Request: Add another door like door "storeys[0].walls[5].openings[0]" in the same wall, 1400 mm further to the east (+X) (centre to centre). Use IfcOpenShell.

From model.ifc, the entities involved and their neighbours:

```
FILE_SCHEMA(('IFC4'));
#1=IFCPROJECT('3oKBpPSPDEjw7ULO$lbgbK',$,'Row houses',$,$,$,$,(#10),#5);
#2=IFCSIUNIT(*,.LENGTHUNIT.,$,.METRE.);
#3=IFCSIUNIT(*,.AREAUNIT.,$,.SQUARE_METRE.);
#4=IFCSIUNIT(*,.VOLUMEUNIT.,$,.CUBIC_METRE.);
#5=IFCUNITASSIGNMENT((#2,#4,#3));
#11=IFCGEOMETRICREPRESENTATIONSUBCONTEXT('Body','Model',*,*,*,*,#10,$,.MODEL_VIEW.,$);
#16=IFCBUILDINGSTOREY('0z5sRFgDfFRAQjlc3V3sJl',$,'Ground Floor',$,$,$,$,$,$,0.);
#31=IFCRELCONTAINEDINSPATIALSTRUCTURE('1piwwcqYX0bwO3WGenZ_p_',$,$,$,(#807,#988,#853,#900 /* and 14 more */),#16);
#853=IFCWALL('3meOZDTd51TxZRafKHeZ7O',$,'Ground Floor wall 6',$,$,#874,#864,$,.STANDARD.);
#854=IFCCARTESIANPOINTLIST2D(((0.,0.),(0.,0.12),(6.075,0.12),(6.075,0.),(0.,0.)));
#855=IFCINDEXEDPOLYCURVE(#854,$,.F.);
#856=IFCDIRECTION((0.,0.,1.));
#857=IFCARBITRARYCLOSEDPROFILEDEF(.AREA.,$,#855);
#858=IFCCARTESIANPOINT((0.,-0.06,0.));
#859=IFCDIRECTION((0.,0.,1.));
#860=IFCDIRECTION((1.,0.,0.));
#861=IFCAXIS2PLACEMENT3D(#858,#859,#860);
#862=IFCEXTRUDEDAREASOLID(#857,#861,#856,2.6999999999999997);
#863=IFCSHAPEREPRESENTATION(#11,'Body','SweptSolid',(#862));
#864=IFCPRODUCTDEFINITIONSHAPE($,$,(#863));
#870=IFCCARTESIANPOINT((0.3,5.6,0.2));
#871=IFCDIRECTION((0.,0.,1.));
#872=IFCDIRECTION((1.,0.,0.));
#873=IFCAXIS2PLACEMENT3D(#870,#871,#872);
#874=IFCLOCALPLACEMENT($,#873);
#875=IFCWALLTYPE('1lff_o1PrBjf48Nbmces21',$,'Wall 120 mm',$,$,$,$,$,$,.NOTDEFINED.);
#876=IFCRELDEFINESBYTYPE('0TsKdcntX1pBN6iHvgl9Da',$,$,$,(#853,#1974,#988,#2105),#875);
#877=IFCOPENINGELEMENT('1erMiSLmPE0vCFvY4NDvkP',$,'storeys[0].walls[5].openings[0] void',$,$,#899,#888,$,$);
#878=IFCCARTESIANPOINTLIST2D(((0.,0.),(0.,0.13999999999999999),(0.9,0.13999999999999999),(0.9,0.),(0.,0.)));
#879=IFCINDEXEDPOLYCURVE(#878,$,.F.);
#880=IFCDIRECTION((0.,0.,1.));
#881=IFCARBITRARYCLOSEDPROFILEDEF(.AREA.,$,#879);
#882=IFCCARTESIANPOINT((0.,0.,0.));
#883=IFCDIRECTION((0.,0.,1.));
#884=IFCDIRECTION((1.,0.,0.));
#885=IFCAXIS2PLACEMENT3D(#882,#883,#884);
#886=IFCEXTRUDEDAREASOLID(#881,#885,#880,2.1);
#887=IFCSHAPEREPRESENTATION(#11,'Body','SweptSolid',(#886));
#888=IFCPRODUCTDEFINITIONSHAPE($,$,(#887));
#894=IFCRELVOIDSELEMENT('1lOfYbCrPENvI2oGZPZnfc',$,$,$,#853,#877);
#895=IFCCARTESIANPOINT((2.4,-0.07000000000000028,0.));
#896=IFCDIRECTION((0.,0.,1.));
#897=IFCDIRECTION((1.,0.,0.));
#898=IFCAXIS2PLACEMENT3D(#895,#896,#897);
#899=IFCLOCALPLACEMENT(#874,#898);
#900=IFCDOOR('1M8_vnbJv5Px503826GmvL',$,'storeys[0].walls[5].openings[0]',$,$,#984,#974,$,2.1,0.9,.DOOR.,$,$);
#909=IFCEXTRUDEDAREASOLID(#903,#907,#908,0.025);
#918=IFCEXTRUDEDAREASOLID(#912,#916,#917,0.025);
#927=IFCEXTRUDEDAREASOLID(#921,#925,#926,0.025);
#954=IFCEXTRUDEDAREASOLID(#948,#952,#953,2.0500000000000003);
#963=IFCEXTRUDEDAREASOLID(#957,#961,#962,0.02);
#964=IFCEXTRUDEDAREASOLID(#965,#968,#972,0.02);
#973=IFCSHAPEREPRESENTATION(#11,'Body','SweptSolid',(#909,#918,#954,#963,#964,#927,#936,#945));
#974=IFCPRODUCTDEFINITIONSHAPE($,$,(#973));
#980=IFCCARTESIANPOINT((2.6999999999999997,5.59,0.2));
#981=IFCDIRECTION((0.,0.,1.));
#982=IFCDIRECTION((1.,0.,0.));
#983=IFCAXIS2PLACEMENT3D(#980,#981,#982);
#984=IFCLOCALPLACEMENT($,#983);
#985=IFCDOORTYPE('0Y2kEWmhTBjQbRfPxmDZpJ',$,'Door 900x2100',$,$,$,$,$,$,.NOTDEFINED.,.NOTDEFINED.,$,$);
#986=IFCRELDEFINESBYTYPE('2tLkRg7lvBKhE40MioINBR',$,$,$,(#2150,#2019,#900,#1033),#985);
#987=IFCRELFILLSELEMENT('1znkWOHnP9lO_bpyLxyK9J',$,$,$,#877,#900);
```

```python
import ifcopenshell
import ifcopenshell.api.feature
import ifcopenshell.api.geometry
import ifcopenshell.api.root
import ifcopenshell.geom
import ifcopenshell.util.element
import ifcopenshell.util.placement
import ifcopenshell.util.shape

model = ifcopenshell.open("model.ifc")
settings = ifcopenshell.geom.settings()


def volume(element):
    """Net volume in cubic metres, openings subtracted."""
    shape = ifcopenshell.geom.create_shape(settings, element)
    return ifcopenshell.util.shape.get_volume(shape.geometry)


door = model.by_guid("1M8_vnbJv5Px503826GmvL")
opening = door.FillsVoids[0].RelatingOpeningElement
wall = opening.VoidsElements[0].RelatingBuildingElement
before = volume(wall)
shift = ifcopenshell.util.placement.get_local_placement(wall.ObjectPlacement)[:3, 0] * 1.4

# copy_class copies the void relationship, type, container and properties, but no geometry.
new_opening = ifcopenshell.api.root.copy_class(model, product=opening)
new_opening.Representation = ifcopenshell.util.element.copy_deep(
    model, opening.Representation, exclude=["IfcGeometricRepresentationContext", "IfcRepresentationMap"]
)
new_door = ifcopenshell.api.root.copy_class(model, product=door)
new_door.Representation = ifcopenshell.util.element.copy_deep(
    model, door.Representation, exclude=["IfcGeometricRepresentationContext", "IfcRepresentationMap"]
)
ifcopenshell.api.feature.add_filling(model, opening=new_opening, element=new_door)

for old, new in ((opening, new_opening), (door, new_door)):
    matrix = ifcopenshell.util.placement.get_local_placement(old.ObjectPlacement)
    matrix[:3, 3] += shift
    ifcopenshell.api.geometry.edit_object_placement(model, product=new, matrix=matrix, is_si=False)

after = volume(wall)

print(f"wall volume {before:.3f} -> {after:.3f} m3")

model.write("model_v2.ifc")
```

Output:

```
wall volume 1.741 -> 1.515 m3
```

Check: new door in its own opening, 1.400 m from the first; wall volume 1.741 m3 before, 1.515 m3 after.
